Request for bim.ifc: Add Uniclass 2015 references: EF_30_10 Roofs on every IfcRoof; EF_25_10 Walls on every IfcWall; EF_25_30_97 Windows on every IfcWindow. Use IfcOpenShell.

First a look at what the model holds.

```python
import ifcopenshell

model = ifcopenshell.open("bim.ifc")
print(model.schema)
print("classifications:", [c.Name for c in model.by_type("IfcClassification")])
for ifc_class in ("IfcDoor", "IfcRoof", "IfcStair", "IfcWall", "IfcWindow"):
    print(ifc_class, len(model.by_type(ifc_class)))
```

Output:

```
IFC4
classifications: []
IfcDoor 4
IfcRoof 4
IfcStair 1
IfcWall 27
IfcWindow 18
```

```python
import ifcopenshell
import ifcopenshell.api.classification

model = ifcopenshell.open("bim.ifc")

system = ifcopenshell.api.classification.add_classification(model, classification="Uniclass 2015")

codes = {
    "IfcRoof": ("EF_30_10", "Roofs"),
    "IfcWall": ("EF_25_10", "Walls"),
    "IfcWindow": ("EF_25_30_97", "Windows"),
}
for ifc_class, (code, name) in codes.items():
    products = model.by_type(ifc_class)
    ifcopenshell.api.classification.add_reference(
        model, products=products, classification=system, identification=code, name=name
    )
    print(code, len(products))

model.write("bim_edited.ifc")
```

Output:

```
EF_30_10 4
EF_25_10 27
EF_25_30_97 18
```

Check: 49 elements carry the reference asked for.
